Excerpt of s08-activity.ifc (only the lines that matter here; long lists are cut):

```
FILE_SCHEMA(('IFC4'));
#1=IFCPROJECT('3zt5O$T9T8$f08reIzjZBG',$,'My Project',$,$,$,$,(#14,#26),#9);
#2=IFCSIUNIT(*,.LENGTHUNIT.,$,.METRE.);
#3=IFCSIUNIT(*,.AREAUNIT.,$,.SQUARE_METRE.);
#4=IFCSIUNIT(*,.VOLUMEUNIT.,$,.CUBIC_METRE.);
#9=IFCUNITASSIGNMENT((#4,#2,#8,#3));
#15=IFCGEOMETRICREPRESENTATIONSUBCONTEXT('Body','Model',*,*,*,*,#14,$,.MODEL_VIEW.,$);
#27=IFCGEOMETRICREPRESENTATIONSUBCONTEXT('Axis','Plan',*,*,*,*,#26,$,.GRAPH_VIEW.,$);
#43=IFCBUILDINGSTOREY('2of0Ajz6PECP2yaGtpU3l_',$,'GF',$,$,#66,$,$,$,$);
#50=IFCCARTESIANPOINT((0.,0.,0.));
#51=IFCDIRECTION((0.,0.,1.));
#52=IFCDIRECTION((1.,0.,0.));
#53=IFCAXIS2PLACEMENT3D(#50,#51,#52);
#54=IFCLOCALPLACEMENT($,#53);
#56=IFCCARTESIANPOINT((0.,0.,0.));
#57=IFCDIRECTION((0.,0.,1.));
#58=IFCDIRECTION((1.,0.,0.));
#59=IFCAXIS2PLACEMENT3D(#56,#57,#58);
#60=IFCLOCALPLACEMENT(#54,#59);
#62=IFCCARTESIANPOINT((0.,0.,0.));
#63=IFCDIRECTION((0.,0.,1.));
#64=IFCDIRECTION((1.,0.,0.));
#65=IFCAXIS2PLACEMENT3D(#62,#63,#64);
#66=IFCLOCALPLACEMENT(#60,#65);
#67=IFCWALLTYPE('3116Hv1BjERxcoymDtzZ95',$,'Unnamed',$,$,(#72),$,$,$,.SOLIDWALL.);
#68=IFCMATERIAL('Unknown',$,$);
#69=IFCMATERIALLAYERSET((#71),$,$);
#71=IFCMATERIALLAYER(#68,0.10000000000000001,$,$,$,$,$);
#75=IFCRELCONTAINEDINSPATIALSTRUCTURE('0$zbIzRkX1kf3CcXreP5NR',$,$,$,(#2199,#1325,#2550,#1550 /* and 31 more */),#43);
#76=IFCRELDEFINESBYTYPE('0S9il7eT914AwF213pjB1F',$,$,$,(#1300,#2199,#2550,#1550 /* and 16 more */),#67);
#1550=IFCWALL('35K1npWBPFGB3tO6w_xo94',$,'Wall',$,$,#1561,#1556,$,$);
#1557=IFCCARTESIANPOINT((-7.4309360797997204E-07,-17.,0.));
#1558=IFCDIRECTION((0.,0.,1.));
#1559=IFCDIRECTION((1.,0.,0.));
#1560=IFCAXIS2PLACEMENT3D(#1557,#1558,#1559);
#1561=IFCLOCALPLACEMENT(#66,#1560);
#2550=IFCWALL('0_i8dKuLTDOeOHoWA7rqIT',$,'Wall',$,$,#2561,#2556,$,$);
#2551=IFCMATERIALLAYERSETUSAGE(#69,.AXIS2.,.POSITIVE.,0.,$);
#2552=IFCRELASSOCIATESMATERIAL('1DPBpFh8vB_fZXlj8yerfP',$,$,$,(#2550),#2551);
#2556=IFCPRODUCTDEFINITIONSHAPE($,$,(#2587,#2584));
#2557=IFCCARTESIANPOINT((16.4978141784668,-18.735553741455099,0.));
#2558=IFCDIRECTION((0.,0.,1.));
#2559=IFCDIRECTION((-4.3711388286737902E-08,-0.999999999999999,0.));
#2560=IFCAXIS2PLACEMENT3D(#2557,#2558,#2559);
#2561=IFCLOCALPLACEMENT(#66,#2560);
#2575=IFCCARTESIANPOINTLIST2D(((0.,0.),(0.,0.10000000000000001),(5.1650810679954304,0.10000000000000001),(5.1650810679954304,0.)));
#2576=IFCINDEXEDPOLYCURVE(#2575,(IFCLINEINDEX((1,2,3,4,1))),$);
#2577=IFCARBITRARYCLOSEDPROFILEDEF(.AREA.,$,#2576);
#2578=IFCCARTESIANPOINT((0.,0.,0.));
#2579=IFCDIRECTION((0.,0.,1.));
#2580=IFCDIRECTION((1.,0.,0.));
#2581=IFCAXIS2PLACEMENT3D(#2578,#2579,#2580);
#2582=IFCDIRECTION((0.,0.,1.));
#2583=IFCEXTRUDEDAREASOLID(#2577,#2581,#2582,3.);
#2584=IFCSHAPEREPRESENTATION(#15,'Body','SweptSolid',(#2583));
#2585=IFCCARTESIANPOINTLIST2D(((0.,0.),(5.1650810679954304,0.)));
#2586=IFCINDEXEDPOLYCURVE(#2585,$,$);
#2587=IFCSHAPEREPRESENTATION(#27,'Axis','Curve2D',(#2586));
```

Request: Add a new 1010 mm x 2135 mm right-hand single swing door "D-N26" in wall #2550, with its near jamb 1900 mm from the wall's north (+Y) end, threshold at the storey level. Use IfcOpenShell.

```python
import numpy as np
import ifcopenshell
import ifcopenshell.api.feature
import ifcopenshell.api.geometry
import ifcopenshell.api.root
import ifcopenshell.api.spatial
import ifcopenshell.geom
import ifcopenshell.util.element
import ifcopenshell.util.placement
import ifcopenshell.util.representation
import ifcopenshell.util.shape
import ifcopenshell.util.unit

model = ifcopenshell.open("s08-activity.ifc")
unit_scale = ifcopenshell.util.unit.calculate_unit_scale(model)
settings = ifcopenshell.geom.settings()


def volume(element):
    """Net volume in cubic metres, openings subtracted."""
    shape = ifcopenshell.geom.create_shape(settings, element)
    return ifcopenshell.util.shape.get_volume(shape.geometry)


wall = model.by_guid("0_i8dKuLTDOeOHoWA7rqIT")
storey = ifcopenshell.util.element.get_container(wall, ifc_class="IfcBuildingStorey")
context = ifcopenshell.util.representation.get_context(model, "Model", "Body", "MODEL_VIEW")
before = volume(wall)

width, height, from_end, sill = 1.01, 2.135, 1.9, 0.0  # metres

# The wall runs along its own X axis, and the end named is its -X end.
wall_shape = ifcopenshell.geom.create_shape(settings, wall)
x, y, z = ifcopenshell.util.shape.get_vertices(wall_shape.geometry).T
start = x.min() + from_end
face, thickness = float(y.min()), float(y.max() - y.min())
wall_matrix = ifcopenshell.util.placement.get_local_placement(wall.ObjectPlacement)
level = ifcopenshell.util.placement.get_local_placement(storey.ObjectPlacement)[2, 3]


def in_wall(x, y):
    """Placement at x, y metres in the wall's axes, at sill height."""
    matrix = wall_matrix.copy()
    matrix[:, 3] = wall_matrix @ np.array([x / unit_scale, y / unit_scale, 0.0, 1.0])
    matrix[2, 3] = level + sill / unit_scale
    return matrix


# Opening: a box that overshoots both wall faces by 50 mm.
opening = ifcopenshell.api.root.create_entity(model, ifc_class="IfcOpeningElement", predefined_type="OPENING")
box = ifcopenshell.api.geometry.add_wall_representation(
    model, context=context, length=width, height=height, thickness=thickness + 0.1
)
ifcopenshell.api.geometry.assign_representation(model, product=opening, representation=box)
ifcopenshell.api.geometry.edit_object_placement(model, product=opening, matrix=in_wall(start, face - 0.05), is_si=False)
ifcopenshell.api.feature.add_feature(model, feature=opening, element=wall)

door = ifcopenshell.api.root.create_entity(model, ifc_class="IfcDoor", name="D-N26", predefined_type="DOOR")
door.OverallWidth, door.OverallHeight = width / unit_scale, height / unit_scale
door.OperationType = "SINGLE_SWING_RIGHT"
body = ifcopenshell.api.geometry.add_door_representation(
    model,
    context=context,
    overall_width=door.OverallWidth,
    overall_height=door.OverallHeight,
    operation_type="SINGLE_SWING_RIGHT",
    lining_properties={"LiningDepth": thickness / unit_scale, "ThresholdDepth": thickness / unit_scale},
)
ifcopenshell.api.geometry.assign_representation(model, product=door, representation=body)
ifcopenshell.api.spatial.assign_container(model, products=[door], relating_structure=storey)
ifcopenshell.api.feature.add_filling(model, opening=opening, element=door)

# The lining spans the wall, so the door starts at the wall face.
ifcopenshell.api.geometry.edit_object_placement(model, product=door, matrix=in_wall(start, face), is_si=False)

after = volume(wall)

print(f"wall volume {before:.3f} -> {after:.3f} m3")

model.write("s08-activity_v2.ifc")
```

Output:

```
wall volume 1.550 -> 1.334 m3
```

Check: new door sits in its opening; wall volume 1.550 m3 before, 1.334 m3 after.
